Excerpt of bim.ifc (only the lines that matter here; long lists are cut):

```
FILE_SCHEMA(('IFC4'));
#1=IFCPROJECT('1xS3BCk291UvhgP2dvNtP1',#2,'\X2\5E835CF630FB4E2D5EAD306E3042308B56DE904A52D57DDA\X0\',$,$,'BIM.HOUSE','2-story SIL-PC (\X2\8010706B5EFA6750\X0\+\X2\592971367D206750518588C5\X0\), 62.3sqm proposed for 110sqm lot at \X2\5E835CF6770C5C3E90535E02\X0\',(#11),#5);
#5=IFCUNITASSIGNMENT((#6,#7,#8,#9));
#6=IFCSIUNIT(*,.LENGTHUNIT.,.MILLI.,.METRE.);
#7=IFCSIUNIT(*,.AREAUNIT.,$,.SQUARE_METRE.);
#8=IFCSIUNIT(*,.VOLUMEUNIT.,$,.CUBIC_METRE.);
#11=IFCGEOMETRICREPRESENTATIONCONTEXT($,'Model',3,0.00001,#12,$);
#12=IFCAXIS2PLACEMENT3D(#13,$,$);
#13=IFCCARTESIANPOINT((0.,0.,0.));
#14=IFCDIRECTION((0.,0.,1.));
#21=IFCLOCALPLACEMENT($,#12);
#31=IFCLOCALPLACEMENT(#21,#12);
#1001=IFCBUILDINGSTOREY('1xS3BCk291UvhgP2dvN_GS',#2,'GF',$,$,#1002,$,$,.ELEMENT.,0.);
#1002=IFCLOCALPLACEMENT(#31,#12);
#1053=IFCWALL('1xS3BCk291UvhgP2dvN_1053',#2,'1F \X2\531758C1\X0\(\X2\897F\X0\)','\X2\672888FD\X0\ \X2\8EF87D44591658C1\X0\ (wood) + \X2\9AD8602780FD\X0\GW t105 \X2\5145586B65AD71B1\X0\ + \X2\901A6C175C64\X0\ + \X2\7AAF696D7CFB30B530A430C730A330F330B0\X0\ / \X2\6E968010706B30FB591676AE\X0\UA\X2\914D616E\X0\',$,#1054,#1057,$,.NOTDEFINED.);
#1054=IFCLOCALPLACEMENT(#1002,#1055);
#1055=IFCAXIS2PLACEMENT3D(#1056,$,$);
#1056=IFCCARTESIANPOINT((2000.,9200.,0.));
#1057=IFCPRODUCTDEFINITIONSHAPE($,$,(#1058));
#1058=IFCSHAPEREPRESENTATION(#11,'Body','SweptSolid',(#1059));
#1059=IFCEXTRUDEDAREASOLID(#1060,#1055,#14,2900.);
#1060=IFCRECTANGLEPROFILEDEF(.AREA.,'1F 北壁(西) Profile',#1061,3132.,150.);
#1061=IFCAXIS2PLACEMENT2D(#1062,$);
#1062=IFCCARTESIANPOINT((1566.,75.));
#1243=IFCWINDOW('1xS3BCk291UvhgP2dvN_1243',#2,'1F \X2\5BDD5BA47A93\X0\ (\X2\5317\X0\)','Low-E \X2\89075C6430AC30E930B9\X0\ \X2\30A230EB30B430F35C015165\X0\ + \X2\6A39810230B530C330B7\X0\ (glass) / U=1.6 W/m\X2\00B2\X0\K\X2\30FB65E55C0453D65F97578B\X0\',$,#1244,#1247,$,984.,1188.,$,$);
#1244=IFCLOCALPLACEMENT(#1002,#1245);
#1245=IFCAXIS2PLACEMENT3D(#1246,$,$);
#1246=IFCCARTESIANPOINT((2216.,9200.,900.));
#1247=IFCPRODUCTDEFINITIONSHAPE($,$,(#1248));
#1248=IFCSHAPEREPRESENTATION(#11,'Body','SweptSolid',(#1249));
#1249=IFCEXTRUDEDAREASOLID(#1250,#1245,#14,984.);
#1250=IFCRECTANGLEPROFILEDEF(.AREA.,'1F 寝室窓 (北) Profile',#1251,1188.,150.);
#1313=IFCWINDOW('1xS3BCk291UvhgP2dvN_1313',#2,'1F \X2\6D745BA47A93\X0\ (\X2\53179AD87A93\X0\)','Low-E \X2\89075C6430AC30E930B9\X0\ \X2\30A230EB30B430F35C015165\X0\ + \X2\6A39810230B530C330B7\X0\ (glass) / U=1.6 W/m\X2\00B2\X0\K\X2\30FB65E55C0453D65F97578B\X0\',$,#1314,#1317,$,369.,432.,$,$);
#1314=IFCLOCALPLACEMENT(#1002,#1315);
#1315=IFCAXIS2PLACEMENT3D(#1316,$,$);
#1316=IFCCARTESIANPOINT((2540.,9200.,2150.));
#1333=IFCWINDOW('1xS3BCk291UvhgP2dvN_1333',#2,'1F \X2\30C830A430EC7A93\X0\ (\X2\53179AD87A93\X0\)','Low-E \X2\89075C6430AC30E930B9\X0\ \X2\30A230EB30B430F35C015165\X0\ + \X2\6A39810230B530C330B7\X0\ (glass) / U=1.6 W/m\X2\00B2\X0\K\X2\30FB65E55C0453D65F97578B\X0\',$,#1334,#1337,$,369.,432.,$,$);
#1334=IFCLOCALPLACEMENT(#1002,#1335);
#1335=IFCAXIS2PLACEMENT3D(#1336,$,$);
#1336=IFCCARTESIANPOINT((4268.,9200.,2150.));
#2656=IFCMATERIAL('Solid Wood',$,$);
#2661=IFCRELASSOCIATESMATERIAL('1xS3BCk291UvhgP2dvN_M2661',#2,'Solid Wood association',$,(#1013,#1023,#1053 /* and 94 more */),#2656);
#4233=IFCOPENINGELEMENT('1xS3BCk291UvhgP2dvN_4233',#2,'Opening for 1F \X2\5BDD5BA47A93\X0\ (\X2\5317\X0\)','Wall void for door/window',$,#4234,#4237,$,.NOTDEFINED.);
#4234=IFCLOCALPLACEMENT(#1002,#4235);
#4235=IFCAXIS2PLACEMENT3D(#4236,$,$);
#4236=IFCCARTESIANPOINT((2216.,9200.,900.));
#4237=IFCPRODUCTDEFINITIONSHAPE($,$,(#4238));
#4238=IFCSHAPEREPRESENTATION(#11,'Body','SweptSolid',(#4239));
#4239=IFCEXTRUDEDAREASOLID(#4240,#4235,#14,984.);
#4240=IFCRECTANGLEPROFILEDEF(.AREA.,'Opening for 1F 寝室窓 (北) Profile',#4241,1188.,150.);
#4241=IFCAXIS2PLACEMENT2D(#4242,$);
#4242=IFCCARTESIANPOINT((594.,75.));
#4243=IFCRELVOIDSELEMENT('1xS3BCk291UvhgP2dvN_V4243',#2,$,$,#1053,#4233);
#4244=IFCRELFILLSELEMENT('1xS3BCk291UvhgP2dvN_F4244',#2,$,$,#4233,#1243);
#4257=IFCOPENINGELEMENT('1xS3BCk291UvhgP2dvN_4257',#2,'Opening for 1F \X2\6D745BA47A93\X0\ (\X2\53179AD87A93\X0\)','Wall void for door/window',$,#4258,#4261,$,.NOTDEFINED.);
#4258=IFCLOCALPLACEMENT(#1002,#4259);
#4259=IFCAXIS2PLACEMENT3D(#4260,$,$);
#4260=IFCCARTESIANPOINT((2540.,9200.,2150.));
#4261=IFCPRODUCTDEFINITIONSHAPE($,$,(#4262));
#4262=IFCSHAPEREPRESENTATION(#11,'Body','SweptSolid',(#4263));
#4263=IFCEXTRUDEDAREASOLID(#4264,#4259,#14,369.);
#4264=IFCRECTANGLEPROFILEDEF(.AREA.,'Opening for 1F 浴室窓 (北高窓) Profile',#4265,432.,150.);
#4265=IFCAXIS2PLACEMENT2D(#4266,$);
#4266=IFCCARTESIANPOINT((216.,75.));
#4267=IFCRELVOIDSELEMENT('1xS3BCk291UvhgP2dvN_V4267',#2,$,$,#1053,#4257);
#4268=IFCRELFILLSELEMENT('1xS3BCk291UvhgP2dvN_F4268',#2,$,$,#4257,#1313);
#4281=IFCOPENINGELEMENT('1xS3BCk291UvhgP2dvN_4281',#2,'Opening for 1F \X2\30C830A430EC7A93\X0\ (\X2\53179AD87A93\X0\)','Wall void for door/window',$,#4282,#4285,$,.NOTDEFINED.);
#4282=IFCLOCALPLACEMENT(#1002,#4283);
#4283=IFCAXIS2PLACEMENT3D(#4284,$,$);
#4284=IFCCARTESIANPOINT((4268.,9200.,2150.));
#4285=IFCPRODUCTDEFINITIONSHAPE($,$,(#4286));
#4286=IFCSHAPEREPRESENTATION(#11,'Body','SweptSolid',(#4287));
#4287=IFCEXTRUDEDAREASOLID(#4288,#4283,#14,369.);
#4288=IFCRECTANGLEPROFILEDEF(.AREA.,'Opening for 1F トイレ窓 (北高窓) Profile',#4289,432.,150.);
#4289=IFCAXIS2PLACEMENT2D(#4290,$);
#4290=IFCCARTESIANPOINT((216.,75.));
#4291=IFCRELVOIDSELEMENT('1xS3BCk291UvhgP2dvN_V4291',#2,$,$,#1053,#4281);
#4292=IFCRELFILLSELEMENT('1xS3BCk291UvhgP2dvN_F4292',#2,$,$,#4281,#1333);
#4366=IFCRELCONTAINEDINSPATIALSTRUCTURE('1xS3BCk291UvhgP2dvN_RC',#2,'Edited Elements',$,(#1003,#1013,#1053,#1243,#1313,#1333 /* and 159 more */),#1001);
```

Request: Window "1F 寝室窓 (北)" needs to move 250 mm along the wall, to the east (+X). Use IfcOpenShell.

```python
import ifcopenshell
import ifcopenshell.api.geometry
import ifcopenshell.util.placement
import ifcopenshell.util.unit

model = ifcopenshell.open("bim.ifc")
unit_scale = ifcopenshell.util.unit.calculate_unit_scale(model)

window = model.by_guid("1xS3BCk291UvhgP2dvN_1243")
opening = window.FillsVoids[0].RelatingOpeningElement
wall = opening.VoidsElements[0].RelatingBuildingElement

wall_matrix = ifcopenshell.util.placement.get_local_placement(wall.ObjectPlacement)
shift = wall_matrix[:3, 0] * 0.25 / unit_scale
before = ifcopenshell.util.placement.get_local_placement(window.ObjectPlacement)[:3, 3].copy()

# The window is not placed relative to its opening, so move both.
for product in (opening, window):
    matrix = ifcopenshell.util.placement.get_local_placement(product.ObjectPlacement)
    matrix[:3, 3] += shift
    ifcopenshell.api.geometry.edit_object_placement(model, product=product, matrix=matrix, is_si=False)

after = ifcopenshell.util.placement.get_local_placement(window.ObjectPlacement)[:3, 3]
print("window moved by", (after - before).round(3) + 0.0)

model.write("bim_edited.ifc")
```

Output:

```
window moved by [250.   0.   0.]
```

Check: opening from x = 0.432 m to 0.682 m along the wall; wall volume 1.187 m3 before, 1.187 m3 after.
